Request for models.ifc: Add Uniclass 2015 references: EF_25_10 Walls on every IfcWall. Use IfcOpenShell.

First a look at what the model holds.

```python
import ifcopenshell

model = ifcopenshell.open("models.ifc")
print(model.schema)
print("classifications:", [c.Name for c in model.by_type("IfcClassification")])
for ifc_class in ("IfcDoor", "IfcRoof", "IfcStair", "IfcWall", "IfcWindow"):
    print(ifc_class, len(model.by_type(ifc_class)))
```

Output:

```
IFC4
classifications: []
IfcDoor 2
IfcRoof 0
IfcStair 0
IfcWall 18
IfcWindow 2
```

```python
import ifcopenshell
import ifcopenshell.api.classification

model = ifcopenshell.open("models.ifc")

system = ifcopenshell.api.classification.add_classification(model, classification="Uniclass 2015")

codes = {
    "IfcWall": ("EF_25_10", "Walls"),
}
for ifc_class, (code, name) in codes.items():
    products = model.by_type(ifc_class)
    ifcopenshell.api.classification.add_reference(
        model, products=products, classification=system, identification=code, name=name
    )
    print(code, len(products))

model.write("models-out.ifc")
```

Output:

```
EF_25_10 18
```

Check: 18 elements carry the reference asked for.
